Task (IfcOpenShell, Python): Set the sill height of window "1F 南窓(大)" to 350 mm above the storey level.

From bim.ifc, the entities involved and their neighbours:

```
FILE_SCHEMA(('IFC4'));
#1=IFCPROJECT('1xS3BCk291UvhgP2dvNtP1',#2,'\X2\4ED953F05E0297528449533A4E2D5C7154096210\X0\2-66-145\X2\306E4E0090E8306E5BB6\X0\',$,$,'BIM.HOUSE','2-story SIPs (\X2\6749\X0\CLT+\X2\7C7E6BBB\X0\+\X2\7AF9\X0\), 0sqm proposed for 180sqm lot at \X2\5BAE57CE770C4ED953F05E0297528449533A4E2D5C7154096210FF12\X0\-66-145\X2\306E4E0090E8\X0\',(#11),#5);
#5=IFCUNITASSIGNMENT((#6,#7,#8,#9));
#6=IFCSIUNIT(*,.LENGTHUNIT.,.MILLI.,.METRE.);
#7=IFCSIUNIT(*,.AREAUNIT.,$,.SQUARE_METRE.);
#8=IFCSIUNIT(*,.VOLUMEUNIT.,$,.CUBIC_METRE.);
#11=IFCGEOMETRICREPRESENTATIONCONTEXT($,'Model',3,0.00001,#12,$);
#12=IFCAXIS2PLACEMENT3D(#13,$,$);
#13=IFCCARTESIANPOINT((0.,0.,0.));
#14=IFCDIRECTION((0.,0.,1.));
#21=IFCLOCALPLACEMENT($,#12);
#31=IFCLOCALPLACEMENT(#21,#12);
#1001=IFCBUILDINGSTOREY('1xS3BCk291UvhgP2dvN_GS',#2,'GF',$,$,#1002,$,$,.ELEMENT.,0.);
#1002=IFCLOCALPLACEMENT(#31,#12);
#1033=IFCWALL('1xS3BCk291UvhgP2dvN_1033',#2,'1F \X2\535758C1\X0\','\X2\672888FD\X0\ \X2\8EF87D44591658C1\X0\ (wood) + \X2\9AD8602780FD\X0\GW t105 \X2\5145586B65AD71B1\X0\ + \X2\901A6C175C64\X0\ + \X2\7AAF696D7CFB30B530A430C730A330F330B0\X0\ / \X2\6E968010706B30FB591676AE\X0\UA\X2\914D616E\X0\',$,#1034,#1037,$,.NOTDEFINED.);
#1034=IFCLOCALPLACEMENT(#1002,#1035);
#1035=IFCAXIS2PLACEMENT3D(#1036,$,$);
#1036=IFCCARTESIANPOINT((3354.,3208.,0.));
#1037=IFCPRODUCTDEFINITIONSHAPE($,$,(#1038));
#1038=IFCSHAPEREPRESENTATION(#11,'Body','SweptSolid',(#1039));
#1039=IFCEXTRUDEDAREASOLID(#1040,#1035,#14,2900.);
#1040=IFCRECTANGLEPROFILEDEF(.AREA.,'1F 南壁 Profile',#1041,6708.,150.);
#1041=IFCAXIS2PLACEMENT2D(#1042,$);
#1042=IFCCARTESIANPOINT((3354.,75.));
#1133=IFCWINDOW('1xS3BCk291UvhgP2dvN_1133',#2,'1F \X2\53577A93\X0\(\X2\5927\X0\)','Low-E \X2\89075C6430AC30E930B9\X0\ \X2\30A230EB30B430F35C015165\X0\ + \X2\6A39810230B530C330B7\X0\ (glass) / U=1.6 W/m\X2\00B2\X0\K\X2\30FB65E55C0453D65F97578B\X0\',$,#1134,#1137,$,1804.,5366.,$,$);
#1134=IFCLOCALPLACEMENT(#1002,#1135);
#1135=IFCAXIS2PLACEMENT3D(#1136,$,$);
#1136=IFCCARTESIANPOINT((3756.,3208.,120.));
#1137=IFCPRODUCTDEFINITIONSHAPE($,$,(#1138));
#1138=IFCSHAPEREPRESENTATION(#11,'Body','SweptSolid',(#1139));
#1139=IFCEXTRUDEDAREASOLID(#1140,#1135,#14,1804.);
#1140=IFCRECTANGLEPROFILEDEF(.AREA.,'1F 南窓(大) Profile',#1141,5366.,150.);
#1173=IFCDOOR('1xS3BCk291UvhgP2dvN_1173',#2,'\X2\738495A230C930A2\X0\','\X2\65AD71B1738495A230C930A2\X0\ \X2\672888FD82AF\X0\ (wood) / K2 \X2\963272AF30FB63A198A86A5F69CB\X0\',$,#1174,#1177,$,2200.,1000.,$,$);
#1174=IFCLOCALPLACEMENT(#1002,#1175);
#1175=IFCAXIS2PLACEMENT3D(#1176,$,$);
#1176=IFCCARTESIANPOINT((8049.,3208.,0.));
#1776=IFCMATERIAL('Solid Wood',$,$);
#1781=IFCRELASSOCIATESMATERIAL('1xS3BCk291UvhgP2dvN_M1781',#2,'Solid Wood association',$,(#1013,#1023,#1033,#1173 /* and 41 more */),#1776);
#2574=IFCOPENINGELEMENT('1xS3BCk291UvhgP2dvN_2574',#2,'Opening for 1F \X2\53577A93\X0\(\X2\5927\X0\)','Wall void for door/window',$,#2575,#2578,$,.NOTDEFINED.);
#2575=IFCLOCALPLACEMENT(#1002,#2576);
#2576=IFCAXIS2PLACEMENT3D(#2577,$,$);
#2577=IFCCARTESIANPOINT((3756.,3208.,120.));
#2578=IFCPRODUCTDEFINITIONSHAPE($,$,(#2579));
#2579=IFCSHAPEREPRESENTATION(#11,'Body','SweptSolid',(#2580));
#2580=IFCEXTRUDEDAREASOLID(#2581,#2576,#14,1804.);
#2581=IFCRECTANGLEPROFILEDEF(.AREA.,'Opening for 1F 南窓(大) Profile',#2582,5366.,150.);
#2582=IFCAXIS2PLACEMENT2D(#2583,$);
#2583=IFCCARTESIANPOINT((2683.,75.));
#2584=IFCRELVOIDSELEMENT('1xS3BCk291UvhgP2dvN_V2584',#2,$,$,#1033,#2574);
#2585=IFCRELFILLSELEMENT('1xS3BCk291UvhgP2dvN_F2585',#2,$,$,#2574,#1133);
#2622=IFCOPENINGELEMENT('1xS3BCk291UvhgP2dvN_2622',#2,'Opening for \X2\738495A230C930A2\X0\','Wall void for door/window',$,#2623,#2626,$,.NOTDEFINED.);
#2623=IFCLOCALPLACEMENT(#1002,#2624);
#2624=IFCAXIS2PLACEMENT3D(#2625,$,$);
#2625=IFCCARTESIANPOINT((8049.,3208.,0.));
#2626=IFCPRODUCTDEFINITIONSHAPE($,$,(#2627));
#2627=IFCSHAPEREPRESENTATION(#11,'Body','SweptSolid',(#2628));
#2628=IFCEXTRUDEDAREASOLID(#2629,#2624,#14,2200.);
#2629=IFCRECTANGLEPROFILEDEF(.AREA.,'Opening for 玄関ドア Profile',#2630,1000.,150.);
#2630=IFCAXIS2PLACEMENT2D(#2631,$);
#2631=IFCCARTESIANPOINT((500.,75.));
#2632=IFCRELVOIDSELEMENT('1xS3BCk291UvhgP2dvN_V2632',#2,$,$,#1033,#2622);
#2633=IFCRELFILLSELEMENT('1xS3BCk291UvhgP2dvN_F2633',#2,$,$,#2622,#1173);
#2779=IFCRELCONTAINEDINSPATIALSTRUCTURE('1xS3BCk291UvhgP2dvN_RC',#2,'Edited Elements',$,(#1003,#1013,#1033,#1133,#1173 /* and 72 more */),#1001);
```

```python
import numpy as np
import ifcopenshell
import ifcopenshell.api.geometry
import ifcopenshell.geom
import ifcopenshell.util.element
import ifcopenshell.util.placement
import ifcopenshell.util.shape
import ifcopenshell.util.unit

model = ifcopenshell.open("bim.ifc")
unit_scale = ifcopenshell.util.unit.calculate_unit_scale(model)

window = model.by_guid("1xS3BCk291UvhgP2dvN_1133")
opening = window.FillsVoids[0].RelatingOpeningElement
storey = ifcopenshell.util.element.get_container(window, ifc_class="IfcBuildingStorey")
level = ifcopenshell.util.placement.get_local_placement(storey.ObjectPlacement)[2, 3]

# The opening's origin need not be at the sill, so measure its lowest point.
shape = ifcopenshell.geom.create_shape(ifcopenshell.geom.settings(), opening)
bottom = ifcopenshell.util.shape.get_shape_bottom_elevation(shape, shape.geometry) / unit_scale
dz = level + 350.0 - bottom

shift = np.array([0.0, 0.0, dz])
# The window is not placed relative to its opening, so move both.
for product in (opening, window):
    matrix = ifcopenshell.util.placement.get_local_placement(product.ObjectPlacement)
    matrix[:3, 3] += shift
    ifcopenshell.api.geometry.edit_object_placement(model, product=product, matrix=matrix, is_si=False)

print(f"moved by {dz * unit_scale:+.3f} m")

model.write("bim-out.ifc")
```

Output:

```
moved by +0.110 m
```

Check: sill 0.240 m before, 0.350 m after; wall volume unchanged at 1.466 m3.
